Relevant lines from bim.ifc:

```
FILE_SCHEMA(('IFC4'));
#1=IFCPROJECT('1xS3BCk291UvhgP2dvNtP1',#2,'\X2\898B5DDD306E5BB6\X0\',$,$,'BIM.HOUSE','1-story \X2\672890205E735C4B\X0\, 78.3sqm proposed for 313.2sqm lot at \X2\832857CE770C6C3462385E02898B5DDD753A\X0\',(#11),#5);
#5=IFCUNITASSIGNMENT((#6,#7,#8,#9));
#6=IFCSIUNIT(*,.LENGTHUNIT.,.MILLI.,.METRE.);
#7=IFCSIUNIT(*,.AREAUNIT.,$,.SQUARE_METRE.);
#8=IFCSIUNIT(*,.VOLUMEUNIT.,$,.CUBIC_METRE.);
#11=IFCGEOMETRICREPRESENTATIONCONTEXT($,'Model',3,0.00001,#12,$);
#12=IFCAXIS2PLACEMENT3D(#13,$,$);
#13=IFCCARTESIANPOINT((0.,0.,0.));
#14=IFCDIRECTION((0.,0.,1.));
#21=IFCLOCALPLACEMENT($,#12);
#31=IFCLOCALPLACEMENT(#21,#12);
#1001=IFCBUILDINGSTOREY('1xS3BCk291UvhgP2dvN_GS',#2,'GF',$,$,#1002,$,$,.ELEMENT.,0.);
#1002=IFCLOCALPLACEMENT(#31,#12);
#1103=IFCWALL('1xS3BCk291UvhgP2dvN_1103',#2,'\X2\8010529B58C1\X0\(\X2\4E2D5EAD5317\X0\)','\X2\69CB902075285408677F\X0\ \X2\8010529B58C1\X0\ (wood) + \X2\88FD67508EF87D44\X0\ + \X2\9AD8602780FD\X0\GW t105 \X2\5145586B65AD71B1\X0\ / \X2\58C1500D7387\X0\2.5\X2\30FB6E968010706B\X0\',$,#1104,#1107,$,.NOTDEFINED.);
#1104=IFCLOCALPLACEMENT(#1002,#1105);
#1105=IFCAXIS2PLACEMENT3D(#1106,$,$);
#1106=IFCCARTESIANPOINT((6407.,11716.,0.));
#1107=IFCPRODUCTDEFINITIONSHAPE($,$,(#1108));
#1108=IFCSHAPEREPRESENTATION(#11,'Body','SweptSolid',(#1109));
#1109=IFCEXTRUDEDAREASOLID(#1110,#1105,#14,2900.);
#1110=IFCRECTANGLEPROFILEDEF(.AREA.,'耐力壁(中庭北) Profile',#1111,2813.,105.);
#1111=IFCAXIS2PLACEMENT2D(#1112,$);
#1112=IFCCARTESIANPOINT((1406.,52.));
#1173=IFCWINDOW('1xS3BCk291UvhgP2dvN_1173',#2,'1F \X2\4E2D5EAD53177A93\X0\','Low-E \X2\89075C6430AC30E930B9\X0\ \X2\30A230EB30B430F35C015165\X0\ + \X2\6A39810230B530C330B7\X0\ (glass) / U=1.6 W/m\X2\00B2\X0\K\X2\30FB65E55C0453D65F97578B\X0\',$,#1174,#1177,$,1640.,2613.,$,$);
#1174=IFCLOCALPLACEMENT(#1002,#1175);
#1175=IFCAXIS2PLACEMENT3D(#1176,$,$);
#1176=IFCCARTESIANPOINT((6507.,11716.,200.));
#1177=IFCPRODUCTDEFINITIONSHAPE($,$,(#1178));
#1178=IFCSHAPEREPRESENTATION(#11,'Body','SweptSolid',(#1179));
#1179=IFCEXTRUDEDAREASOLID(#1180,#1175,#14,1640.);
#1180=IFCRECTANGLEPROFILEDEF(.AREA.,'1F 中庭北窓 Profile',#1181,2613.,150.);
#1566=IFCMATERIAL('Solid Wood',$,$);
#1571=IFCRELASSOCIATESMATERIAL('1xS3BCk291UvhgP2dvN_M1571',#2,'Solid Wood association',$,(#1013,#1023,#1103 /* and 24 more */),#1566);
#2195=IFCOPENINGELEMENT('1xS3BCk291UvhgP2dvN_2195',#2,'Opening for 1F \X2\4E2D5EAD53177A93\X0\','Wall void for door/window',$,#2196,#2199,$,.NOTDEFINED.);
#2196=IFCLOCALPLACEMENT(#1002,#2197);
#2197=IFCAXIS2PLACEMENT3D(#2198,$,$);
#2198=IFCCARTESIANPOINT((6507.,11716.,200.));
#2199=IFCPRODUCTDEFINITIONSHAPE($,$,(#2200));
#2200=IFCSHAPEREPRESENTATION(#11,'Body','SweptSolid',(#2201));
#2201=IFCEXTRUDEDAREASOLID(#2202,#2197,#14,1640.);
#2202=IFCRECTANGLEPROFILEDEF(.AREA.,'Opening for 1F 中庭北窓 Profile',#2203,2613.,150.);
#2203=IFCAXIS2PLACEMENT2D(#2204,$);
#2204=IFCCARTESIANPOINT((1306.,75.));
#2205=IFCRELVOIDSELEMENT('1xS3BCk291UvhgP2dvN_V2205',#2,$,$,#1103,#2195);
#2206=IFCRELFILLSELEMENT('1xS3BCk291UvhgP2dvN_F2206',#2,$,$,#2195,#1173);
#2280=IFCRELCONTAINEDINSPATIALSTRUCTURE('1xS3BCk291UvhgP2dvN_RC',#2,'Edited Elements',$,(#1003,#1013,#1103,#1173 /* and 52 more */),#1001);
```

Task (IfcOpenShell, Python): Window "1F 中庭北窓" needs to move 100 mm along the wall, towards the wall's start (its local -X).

```python
import ifcopenshell
import ifcopenshell.api.geometry
import ifcopenshell.util.placement
import ifcopenshell.util.unit

model = ifcopenshell.open("bim.ifc")
unit_scale = ifcopenshell.util.unit.calculate_unit_scale(model)

window = model.by_guid("1xS3BCk291UvhgP2dvN_1173")
opening = window.FillsVoids[0].RelatingOpeningElement
wall = opening.VoidsElements[0].RelatingBuildingElement

wall_matrix = ifcopenshell.util.placement.get_local_placement(wall.ObjectPlacement)
shift = wall_matrix[:3, 0] * -0.1 / unit_scale
before = ifcopenshell.util.placement.get_local_placement(window.ObjectPlacement)[:3, 3].copy()

# The window is not placed relative to its opening, so move both.
for product in (opening, window):
    matrix = ifcopenshell.util.placement.get_local_placement(product.ObjectPlacement)
    matrix[:3, 3] += shift
    ifcopenshell.api.geometry.edit_object_placement(model, product=product, matrix=matrix, is_si=False)

after = ifcopenshell.util.placement.get_local_placement(window.ObjectPlacement)[:3, 3]
print("window moved by", (after - before).round(3) + 0.0)

model.write("bim_edited.ifc")
```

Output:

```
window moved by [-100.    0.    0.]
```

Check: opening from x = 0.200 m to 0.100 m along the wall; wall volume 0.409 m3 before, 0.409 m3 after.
